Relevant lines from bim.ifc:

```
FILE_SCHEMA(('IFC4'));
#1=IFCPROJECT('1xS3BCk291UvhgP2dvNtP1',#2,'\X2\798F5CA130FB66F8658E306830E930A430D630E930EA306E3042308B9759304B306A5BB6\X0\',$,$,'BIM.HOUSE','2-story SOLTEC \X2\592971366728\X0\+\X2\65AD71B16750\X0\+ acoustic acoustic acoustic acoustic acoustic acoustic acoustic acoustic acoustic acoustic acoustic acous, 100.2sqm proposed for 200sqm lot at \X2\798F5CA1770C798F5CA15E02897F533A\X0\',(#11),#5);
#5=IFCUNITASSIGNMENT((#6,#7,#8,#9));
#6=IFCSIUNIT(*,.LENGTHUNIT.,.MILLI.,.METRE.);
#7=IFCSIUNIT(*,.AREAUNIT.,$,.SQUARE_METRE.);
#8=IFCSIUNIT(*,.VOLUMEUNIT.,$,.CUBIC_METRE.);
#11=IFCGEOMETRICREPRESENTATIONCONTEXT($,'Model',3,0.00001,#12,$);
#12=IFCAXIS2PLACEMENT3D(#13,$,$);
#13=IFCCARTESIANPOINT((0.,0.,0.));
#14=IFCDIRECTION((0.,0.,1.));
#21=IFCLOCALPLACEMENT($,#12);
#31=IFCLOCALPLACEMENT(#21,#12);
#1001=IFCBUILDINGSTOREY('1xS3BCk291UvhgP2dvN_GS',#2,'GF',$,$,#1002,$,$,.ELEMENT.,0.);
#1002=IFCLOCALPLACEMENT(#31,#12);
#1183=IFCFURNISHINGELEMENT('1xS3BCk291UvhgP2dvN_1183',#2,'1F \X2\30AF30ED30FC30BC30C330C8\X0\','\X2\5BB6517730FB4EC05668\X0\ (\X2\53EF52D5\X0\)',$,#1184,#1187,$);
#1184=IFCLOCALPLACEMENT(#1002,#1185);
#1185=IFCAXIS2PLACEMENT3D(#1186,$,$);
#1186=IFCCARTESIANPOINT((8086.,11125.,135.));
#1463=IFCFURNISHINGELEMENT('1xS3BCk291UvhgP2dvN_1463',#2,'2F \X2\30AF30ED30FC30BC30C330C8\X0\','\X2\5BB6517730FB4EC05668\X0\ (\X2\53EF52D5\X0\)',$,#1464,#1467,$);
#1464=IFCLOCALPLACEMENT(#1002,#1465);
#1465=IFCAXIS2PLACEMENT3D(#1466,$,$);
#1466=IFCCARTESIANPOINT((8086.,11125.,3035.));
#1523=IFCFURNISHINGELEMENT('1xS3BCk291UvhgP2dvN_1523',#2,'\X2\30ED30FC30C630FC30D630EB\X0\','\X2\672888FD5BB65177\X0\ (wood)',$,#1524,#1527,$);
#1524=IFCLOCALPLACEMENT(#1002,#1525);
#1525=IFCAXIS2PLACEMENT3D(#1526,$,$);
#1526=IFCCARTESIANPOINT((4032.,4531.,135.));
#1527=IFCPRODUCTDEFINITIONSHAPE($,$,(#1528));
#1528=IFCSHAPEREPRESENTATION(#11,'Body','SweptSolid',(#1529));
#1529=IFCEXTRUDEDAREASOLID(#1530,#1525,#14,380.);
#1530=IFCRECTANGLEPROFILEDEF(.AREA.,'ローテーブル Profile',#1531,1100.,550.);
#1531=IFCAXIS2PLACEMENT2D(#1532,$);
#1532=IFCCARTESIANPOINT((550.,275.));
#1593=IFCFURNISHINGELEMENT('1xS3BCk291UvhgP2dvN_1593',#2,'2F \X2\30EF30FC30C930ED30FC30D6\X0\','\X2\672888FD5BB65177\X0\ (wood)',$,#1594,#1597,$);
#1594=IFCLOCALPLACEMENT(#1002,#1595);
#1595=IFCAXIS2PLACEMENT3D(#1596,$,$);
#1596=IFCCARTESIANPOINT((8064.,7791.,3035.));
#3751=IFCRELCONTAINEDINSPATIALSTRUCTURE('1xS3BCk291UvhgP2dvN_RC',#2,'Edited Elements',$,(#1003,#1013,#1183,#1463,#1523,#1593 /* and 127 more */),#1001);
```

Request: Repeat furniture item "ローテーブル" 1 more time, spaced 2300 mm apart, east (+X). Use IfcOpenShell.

```python
import numpy as np
import ifcopenshell
import ifcopenshell.api.geometry
import ifcopenshell.api.root
import ifcopenshell.util.element
import ifcopenshell.util.placement
import ifcopenshell.util.unit

model = ifcopenshell.open("bim.ifc")
unit_scale = ifcopenshell.util.unit.calculate_unit_scale(model)


def reuse_history(source, copy):
    """copy_class also copies each property set's owner history, people and application; keep the originals."""
    for rel in copy.IsDefinedBy:
        if rel.is_a("IfcRelDefinesByProperties") and (history := rel.RelatingPropertyDefinition.OwnerHistory):
            rel.RelatingPropertyDefinition.OwnerHistory = source.OwnerHistory
            ifcopenshell.util.element.remove_deep2(model, history)


source = model.by_guid("1xS3BCk291UvhgP2dvN_1523")
base = ifcopenshell.util.placement.get_local_placement(source.ObjectPlacement)
step = np.array([1.0, 0.0, 0.0]) * 2.3 / unit_scale

for i in range(1, 2):
    copy = ifcopenshell.api.root.copy_class(model, product=source)
    copy.Representation = ifcopenshell.util.element.copy_deep(
        model, source.Representation, exclude=["IfcGeometricRepresentationContext", "IfcRepresentationMap"]
    )
    reuse_history(source, copy)
    matrix = base.copy()
    matrix[:3, 3] += i * step
    print("added at", matrix[:3, 3].round(3) + 0.0)
    ifcopenshell.api.geometry.edit_object_placement(model, product=copy, matrix=matrix, is_si=False)

model.write("bim_rev.ifc")
```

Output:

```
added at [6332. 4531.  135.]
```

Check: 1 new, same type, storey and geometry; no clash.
